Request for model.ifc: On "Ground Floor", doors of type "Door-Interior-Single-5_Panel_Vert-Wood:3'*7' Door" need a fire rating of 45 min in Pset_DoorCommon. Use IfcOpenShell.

First a look at what the model holds.

```python
import ifcopenshell
import ifcopenshell.util.element

model = ifcopenshell.open("model.ifc")
print(model.schema)
storey = next(s for s in model.by_type("IfcBuildingStorey") if s.Name == "Ground Floor")
doors = [e for e in ifcopenshell.util.element.get_decomposition(storey) if e.is_a("IfcDoor")]
seen = {}
for e in doors:
    element_type = ifcopenshell.util.element.get_type(e)
    key = (element_type.Name if element_type != e and element_type else None, ifcopenshell.util.element.get_pset(e, "Pset_DoorCommon", "FireRating"))
    seen[key] = seen.get(key, 0) + 1
for (name, value), count in sorted(seen.items(), key=str):
    print(count, "x", name, "|", value)
```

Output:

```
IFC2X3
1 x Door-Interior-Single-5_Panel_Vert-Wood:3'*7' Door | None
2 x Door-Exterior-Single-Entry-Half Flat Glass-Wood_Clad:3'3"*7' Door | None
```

```python
import ifcopenshell
import ifcopenshell.api.pset
import ifcopenshell.util.element

model = ifcopenshell.open("model.ifc")

storey = next(s for s in model.by_type("IfcBuildingStorey") if s.Name == "Ground Floor")
doors = [e for e in ifcopenshell.util.element.get_decomposition(storey) if e.is_a("IfcDoor")]

count = 0
for e in doors:
    element_type = ifcopenshell.util.element.get_type(e)
    if element_type in (None, e) or element_type.Name != "Door-Interior-Single-5_Panel_Vert-Wood:3'*7' Door":
        continue
    # add_pset returns the element's existing set when there is one.
    pset = ifcopenshell.api.pset.add_pset(model, product=e, name="Pset_DoorCommon")
    ifcopenshell.api.pset.edit_pset(model, pset=pset, properties={"FireRating": "45 min"})
    count += 1

print(count, "doors updated")

model.write("model_v2.ifc")
```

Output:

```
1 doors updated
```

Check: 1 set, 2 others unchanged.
